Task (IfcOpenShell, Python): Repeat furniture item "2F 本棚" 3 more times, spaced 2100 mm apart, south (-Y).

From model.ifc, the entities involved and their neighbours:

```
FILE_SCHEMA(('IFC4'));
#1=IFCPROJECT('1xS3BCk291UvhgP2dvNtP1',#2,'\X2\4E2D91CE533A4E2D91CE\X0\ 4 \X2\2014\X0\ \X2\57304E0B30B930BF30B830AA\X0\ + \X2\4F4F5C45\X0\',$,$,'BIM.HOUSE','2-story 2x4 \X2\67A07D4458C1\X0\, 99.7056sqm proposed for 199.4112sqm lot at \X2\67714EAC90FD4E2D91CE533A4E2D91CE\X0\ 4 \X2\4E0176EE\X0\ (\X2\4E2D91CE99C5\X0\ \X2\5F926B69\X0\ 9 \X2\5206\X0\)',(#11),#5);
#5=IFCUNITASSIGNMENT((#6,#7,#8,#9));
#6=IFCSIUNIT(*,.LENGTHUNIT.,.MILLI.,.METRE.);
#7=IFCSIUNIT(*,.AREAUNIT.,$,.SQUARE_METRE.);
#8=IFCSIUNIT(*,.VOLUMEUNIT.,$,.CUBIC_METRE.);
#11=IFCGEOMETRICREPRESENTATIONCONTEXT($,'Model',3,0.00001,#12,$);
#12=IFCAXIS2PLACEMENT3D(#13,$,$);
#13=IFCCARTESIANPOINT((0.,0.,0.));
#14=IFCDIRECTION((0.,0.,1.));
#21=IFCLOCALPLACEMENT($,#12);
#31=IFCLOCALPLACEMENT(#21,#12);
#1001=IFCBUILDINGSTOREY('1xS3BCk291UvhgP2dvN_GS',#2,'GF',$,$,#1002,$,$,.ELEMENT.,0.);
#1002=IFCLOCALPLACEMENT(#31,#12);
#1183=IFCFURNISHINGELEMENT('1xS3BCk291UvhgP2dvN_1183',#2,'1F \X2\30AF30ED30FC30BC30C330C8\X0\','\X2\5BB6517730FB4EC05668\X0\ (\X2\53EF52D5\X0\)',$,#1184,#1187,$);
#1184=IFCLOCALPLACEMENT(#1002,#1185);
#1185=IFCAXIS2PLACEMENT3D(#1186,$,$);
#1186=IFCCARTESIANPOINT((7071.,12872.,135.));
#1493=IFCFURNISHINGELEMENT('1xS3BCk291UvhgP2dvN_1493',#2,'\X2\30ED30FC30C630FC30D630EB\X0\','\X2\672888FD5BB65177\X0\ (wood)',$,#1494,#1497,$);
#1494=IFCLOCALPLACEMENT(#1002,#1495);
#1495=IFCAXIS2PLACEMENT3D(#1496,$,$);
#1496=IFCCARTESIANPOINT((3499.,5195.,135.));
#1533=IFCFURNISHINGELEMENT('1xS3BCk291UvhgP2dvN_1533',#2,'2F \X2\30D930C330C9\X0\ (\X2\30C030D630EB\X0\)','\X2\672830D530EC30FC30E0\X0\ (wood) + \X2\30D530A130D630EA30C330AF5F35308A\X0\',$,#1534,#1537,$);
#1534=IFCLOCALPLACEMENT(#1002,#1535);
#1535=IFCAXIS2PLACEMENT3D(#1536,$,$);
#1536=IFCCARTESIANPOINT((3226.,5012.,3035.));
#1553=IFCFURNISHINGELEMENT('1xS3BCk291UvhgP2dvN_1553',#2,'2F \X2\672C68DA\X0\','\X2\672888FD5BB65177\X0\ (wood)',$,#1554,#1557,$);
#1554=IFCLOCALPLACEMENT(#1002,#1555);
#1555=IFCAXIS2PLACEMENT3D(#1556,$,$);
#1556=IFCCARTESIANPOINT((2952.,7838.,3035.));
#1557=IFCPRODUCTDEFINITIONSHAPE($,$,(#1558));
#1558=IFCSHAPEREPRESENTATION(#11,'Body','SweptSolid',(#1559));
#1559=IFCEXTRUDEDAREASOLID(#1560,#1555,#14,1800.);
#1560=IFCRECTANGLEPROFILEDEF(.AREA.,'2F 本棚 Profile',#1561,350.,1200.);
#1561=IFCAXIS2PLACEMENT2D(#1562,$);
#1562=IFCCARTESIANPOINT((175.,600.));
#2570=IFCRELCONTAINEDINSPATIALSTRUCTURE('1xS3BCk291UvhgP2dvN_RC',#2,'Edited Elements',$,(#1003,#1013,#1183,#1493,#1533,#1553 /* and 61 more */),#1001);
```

```python
import numpy as np
import ifcopenshell
import ifcopenshell.api.geometry
import ifcopenshell.api.root
import ifcopenshell.util.element
import ifcopenshell.util.placement

model = ifcopenshell.open("model.ifc")


def reuse_history(source, copy):
    """copy_class also copies each property set's owner history, people and application; keep the originals."""
    for rel in copy.IsDefinedBy:
        if rel.is_a("IfcRelDefinesByProperties") and (history := rel.RelatingPropertyDefinition.OwnerHistory):
            rel.RelatingPropertyDefinition.OwnerHistory = source.OwnerHistory
            ifcopenshell.util.element.remove_deep2(model, history)


source = model.by_guid("1xS3BCk291UvhgP2dvN_1553")
base = ifcopenshell.util.placement.get_local_placement(source.ObjectPlacement)
step = np.array([0.0, -1.0, 0.0]) * 2100.0

for i in range(1, 4):
    copy = ifcopenshell.api.root.copy_class(model, product=source)
    copy.Representation = ifcopenshell.util.element.copy_deep(
        model, source.Representation, exclude=["IfcGeometricRepresentationContext", "IfcRepresentationMap"]
    )
    reuse_history(source, copy)
    matrix = base.copy()
    matrix[:3, 3] += i * step
    print("added at", matrix[:3, 3].round(3) + 0.0)
    ifcopenshell.api.geometry.edit_object_placement(model, product=copy, matrix=matrix, is_si=False)

model.write("model-out.ifc")
```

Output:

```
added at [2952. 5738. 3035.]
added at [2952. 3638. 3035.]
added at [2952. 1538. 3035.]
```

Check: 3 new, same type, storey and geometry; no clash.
